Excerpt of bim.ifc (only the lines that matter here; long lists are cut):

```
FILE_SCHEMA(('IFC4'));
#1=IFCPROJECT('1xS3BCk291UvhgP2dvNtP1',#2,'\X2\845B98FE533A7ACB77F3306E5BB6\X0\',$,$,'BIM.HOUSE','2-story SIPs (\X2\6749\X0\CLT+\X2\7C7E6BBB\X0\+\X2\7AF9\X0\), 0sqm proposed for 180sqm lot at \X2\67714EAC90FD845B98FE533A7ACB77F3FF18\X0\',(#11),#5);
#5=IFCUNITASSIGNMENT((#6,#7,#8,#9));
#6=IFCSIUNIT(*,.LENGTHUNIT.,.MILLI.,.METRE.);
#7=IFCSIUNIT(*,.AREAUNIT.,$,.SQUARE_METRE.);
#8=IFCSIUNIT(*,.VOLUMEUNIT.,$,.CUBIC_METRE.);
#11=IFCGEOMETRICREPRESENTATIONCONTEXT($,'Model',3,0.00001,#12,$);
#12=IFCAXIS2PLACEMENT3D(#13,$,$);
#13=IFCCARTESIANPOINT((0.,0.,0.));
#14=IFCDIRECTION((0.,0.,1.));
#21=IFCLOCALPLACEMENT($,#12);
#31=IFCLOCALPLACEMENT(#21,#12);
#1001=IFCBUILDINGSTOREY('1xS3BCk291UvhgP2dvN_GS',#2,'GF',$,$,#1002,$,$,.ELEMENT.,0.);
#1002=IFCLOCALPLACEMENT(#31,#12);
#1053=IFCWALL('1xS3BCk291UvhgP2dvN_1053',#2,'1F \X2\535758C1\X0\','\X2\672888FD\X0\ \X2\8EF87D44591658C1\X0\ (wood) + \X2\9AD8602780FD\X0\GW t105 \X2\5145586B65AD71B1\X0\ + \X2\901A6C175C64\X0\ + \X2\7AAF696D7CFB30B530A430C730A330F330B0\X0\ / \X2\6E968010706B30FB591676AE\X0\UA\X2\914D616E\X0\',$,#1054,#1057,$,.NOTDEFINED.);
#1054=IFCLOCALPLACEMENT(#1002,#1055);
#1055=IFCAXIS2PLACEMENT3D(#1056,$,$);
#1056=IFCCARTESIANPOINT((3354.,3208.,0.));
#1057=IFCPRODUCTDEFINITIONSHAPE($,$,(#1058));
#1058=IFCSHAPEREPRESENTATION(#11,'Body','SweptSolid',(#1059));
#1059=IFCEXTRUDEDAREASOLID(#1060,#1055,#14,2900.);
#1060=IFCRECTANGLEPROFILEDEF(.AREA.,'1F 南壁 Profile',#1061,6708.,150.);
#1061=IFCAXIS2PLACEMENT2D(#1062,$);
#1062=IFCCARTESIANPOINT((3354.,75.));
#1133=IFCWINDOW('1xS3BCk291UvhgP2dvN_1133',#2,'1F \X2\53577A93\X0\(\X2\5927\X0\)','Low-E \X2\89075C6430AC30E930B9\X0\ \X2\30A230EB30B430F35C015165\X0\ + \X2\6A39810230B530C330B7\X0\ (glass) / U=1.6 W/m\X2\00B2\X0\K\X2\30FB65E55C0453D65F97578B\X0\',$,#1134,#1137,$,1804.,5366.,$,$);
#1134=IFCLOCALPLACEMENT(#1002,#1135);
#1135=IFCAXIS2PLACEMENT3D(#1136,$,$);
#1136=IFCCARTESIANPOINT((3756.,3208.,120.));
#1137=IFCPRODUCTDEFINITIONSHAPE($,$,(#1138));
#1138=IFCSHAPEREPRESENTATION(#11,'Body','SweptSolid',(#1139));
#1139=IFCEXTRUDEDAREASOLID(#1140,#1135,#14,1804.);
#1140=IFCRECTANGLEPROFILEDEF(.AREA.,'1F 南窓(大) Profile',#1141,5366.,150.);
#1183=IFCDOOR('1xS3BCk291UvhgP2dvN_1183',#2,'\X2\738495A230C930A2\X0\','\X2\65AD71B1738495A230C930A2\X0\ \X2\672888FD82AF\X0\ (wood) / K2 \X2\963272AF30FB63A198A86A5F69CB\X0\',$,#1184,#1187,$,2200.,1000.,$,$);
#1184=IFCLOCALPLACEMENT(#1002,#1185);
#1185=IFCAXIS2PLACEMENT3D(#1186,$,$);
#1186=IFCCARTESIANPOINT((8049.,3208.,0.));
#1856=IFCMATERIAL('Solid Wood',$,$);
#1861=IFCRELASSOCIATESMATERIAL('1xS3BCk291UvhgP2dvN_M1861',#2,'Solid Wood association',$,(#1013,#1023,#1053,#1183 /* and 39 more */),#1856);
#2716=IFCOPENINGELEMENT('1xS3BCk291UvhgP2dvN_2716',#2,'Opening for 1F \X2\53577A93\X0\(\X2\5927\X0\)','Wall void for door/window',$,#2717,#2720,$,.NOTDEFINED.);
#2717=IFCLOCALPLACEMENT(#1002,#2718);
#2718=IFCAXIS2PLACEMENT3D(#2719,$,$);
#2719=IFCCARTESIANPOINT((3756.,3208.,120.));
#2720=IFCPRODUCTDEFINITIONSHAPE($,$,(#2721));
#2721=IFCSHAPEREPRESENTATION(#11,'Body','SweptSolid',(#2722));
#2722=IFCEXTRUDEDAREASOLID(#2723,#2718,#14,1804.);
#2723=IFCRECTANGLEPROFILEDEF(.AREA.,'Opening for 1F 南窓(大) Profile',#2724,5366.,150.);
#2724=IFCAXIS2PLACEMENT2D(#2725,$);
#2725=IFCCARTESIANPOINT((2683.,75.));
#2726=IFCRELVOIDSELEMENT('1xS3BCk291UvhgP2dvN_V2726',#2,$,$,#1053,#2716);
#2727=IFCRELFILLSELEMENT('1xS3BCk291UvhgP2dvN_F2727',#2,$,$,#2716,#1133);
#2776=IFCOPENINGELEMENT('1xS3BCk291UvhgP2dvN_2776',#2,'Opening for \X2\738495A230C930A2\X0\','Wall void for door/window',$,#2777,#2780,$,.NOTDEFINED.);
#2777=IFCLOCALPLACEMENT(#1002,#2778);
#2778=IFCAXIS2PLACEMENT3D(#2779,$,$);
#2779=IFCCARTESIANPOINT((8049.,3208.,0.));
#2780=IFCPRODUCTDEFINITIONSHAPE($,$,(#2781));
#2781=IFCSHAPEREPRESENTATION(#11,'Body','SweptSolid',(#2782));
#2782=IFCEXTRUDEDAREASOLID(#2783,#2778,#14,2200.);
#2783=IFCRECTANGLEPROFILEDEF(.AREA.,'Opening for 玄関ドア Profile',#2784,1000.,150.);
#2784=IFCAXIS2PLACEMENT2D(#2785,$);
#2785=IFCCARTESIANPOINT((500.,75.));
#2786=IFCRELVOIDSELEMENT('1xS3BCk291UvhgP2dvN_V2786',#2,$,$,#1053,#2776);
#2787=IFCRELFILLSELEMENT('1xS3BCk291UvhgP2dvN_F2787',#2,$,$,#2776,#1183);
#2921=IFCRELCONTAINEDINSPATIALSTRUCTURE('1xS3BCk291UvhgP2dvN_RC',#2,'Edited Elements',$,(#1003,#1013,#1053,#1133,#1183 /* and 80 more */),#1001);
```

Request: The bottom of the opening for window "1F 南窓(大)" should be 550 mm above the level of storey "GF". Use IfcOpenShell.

```python
import numpy as np
import ifcopenshell
import ifcopenshell.api.geometry
import ifcopenshell.geom
import ifcopenshell.util.element
import ifcopenshell.util.placement
import ifcopenshell.util.shape
import ifcopenshell.util.unit

model = ifcopenshell.open("bim.ifc")
unit_scale = ifcopenshell.util.unit.calculate_unit_scale(model)

window = model.by_guid("1xS3BCk291UvhgP2dvN_1133")
opening = window.FillsVoids[0].RelatingOpeningElement
storey = ifcopenshell.util.element.get_container(window, ifc_class="IfcBuildingStorey")
level = ifcopenshell.util.placement.get_local_placement(storey.ObjectPlacement)[2, 3]

# The opening's origin need not be at the sill, so measure its lowest point.
shape = ifcopenshell.geom.create_shape(ifcopenshell.geom.settings(), opening)
bottom = ifcopenshell.util.shape.get_shape_bottom_elevation(shape, shape.geometry) / unit_scale
dz = level + 550.0 - bottom

shift = np.array([0.0, 0.0, dz])
# The window is not placed relative to its opening, so move both.
for product in (opening, window):
    matrix = ifcopenshell.util.placement.get_local_placement(product.ObjectPlacement)
    matrix[:3, 3] += shift
    ifcopenshell.api.geometry.edit_object_placement(model, product=product, matrix=matrix, is_si=False)

print(f"moved by {dz * unit_scale:+.3f} m")

model.write("bim-out.ifc")
```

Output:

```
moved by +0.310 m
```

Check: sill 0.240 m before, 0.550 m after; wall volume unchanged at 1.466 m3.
